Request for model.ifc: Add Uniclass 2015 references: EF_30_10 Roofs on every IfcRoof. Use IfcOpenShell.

First a look at what the model holds.

```python
import ifcopenshell

model = ifcopenshell.open("model.ifc")
print(model.schema)
print("classifications:", [c.Name for c in model.by_type("IfcClassification")])
for ifc_class in ("IfcDoor", "IfcRoof", "IfcStair", "IfcWall", "IfcWindow"):
    print(ifc_class, len(model.by_type(ifc_class)))
```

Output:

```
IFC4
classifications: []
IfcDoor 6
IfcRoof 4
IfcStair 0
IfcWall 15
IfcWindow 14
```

```python
import ifcopenshell
import ifcopenshell.api.classification

model = ifcopenshell.open("model.ifc")

system = ifcopenshell.api.classification.add_classification(model, classification="Uniclass 2015")

codes = {
    "IfcRoof": ("EF_30_10", "Roofs"),
}
for ifc_class, (code, name) in codes.items():
    products = model.by_type(ifc_class)
    ifcopenshell.api.classification.add_reference(
        model, products=products, classification=system, identification=code, name=name
    )
    print(code, len(products))

model.write("model_rev.ifc")
```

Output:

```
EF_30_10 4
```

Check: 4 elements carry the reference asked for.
